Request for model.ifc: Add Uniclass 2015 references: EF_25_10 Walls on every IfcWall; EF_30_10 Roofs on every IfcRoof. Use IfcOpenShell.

First a look at what the model holds.

```python
import ifcopenshell

model = ifcopenshell.open("model.ifc")
print(model.schema)
print("classifications:", [c.Name for c in model.by_type("IfcClassification")])
for ifc_class in ("IfcDoor", "IfcRoof", "IfcStair", "IfcWall", "IfcWindow"):
    print(ifc_class, len(model.by_type(ifc_class)))
```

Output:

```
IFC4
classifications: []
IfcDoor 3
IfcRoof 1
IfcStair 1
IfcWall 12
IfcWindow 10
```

```python
import ifcopenshell
import ifcopenshell.api.classification

model = ifcopenshell.open("model.ifc")

system = ifcopenshell.api.classification.add_classification(model, classification="Uniclass 2015")

codes = {
    "IfcWall": ("EF_25_10", "Walls"),
    "IfcRoof": ("EF_30_10", "Roofs"),
}
for ifc_class, (code, name) in codes.items():
    products = model.by_type(ifc_class)
    ifcopenshell.api.classification.add_reference(
        model, products=products, classification=system, identification=code, name=name
    )
    print(code, len(products))

model.write("model_updated.ifc")
```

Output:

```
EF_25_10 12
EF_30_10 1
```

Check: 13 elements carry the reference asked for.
